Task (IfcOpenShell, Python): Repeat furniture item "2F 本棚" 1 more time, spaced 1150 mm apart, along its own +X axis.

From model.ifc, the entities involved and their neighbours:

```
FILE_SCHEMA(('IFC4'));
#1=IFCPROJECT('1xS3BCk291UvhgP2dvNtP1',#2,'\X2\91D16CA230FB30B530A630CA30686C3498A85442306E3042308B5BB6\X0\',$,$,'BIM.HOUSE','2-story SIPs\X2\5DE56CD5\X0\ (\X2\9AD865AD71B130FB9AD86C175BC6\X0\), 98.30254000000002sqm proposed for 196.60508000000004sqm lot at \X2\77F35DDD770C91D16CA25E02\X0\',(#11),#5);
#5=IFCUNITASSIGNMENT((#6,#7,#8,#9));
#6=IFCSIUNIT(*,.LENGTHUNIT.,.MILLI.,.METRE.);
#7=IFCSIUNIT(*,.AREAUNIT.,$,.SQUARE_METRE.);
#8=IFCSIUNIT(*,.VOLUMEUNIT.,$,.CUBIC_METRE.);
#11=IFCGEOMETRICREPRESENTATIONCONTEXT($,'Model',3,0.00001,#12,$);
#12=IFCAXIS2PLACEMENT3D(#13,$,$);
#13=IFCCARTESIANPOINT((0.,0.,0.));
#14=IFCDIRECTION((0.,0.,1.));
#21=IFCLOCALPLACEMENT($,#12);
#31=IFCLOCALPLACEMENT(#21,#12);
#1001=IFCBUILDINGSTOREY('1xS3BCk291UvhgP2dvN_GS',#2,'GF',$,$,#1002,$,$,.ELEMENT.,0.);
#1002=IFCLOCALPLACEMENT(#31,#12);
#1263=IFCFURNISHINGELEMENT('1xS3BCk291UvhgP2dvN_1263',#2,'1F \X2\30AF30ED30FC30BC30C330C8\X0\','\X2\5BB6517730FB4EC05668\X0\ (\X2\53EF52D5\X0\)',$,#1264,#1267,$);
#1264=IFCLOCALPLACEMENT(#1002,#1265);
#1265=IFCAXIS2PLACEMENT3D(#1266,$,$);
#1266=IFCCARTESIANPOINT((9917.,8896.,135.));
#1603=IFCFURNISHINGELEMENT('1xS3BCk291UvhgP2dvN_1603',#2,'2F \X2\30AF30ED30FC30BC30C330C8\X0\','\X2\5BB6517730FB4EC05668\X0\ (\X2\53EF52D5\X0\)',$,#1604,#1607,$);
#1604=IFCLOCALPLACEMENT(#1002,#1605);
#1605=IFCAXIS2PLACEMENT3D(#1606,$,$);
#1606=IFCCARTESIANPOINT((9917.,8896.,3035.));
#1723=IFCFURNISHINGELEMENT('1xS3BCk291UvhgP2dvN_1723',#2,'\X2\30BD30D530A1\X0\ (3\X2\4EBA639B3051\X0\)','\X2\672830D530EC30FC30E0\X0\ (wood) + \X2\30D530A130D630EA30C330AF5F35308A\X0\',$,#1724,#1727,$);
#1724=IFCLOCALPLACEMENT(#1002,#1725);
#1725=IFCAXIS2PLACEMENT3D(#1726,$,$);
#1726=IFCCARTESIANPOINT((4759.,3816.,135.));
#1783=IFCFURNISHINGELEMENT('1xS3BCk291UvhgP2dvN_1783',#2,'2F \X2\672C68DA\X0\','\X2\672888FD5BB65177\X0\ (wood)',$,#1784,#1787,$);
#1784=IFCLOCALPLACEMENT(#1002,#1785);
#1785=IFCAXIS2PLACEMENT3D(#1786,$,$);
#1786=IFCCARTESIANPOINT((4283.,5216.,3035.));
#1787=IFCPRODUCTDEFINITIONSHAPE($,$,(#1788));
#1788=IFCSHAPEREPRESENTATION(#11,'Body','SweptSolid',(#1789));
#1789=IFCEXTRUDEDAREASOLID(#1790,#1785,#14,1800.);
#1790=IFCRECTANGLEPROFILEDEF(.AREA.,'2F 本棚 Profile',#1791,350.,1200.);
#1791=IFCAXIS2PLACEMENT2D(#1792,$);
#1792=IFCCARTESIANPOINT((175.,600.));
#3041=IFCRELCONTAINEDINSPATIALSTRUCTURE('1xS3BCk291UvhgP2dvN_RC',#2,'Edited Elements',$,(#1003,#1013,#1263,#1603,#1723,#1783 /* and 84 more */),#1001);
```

```python
import ifcopenshell
import ifcopenshell.api.geometry
import ifcopenshell.api.root
import ifcopenshell.util.element
import ifcopenshell.util.placement

model = ifcopenshell.open("model.ifc")


def reuse_history(source, copy):
    """copy_class also copies each property set's owner history, people and application; keep the originals."""
    for rel in copy.IsDefinedBy:
        if rel.is_a("IfcRelDefinesByProperties") and (history := rel.RelatingPropertyDefinition.OwnerHistory):
            rel.RelatingPropertyDefinition.OwnerHistory = source.OwnerHistory
            ifcopenshell.util.element.remove_deep2(model, history)


source = model.by_guid("1xS3BCk291UvhgP2dvN_1783")
base = ifcopenshell.util.placement.get_local_placement(source.ObjectPlacement)
step = base[:3, 0] * 1150.0

for i in range(1, 2):
    copy = ifcopenshell.api.root.copy_class(model, product=source)
    copy.Representation = ifcopenshell.util.element.copy_deep(
        model, source.Representation, exclude=["IfcGeometricRepresentationContext", "IfcRepresentationMap"]
    )
    reuse_history(source, copy)
    matrix = base.copy()
    matrix[:3, 3] += i * step
    print("added at", matrix[:3, 3].round(3) + 0.0)
    ifcopenshell.api.geometry.edit_object_placement(model, product=copy, matrix=matrix, is_si=False)

model.write("model-out.ifc")
```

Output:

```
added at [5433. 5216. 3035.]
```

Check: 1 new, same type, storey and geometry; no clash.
